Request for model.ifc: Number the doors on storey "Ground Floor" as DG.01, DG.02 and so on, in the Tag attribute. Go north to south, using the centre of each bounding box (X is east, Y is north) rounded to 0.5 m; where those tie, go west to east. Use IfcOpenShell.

First a look at what the model holds.

```python
import ifcopenshell
import ifcopenshell.util.element
import ifcopenshell.util.placement

model = ifcopenshell.open("model.ifc")
print(model.schema)
storey = next(s for s in model.by_type("IfcBuildingStorey") if s.Name == "Ground Floor")
doors = [e for e in ifcopenshell.util.element.get_decomposition(storey) if e.is_a("IfcDoor")]
for e in sorted(doors, key=lambda e: e.id()):
    origin = ifcopenshell.util.placement.get_local_placement(e.ObjectPlacement)[:3, 3]
    print(e.id(), e.Tag, e.Name, origin.round(2) + 0.0, sep=" | ")
```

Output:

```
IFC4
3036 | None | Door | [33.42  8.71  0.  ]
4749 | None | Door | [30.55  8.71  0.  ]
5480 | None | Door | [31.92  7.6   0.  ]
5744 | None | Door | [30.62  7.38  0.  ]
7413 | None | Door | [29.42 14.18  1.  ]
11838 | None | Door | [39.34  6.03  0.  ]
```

```python
import ifcopenshell
import ifcopenshell.geom
import ifcopenshell.util.element
import ifcopenshell.util.shape

model = ifcopenshell.open("model.ifc")
settings = ifcopenshell.geom.settings()
settings.set("use-world-coords", True)


def centre(element):
    shape = ifcopenshell.geom.create_shape(settings, element)
    return ifcopenshell.util.shape.get_bbox_centroid(shape.geometry)


storey = next(s for s in model.by_type("IfcBuildingStorey") if s.Name == "Ground Floor")
doors = [e for e in ifcopenshell.util.element.get_decomposition(storey) if e.is_a("IfcDoor")]

# Insertion points can sit at a corner or the storey origin, so sort by the geometry (in metres).
centres = {e: centre(e) for e in doors}
doors.sort(key=lambda e: (-round(centres[e][1] / 0.5), centres[e][0]))

for i, e in enumerate(doors, start=1):
    number = f"DG.{i:02d}"
    e.Tag = number
    print(e.id(), number)

model.write("model-out.ifc")
```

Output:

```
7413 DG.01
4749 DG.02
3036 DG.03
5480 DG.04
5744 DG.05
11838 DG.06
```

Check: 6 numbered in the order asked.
